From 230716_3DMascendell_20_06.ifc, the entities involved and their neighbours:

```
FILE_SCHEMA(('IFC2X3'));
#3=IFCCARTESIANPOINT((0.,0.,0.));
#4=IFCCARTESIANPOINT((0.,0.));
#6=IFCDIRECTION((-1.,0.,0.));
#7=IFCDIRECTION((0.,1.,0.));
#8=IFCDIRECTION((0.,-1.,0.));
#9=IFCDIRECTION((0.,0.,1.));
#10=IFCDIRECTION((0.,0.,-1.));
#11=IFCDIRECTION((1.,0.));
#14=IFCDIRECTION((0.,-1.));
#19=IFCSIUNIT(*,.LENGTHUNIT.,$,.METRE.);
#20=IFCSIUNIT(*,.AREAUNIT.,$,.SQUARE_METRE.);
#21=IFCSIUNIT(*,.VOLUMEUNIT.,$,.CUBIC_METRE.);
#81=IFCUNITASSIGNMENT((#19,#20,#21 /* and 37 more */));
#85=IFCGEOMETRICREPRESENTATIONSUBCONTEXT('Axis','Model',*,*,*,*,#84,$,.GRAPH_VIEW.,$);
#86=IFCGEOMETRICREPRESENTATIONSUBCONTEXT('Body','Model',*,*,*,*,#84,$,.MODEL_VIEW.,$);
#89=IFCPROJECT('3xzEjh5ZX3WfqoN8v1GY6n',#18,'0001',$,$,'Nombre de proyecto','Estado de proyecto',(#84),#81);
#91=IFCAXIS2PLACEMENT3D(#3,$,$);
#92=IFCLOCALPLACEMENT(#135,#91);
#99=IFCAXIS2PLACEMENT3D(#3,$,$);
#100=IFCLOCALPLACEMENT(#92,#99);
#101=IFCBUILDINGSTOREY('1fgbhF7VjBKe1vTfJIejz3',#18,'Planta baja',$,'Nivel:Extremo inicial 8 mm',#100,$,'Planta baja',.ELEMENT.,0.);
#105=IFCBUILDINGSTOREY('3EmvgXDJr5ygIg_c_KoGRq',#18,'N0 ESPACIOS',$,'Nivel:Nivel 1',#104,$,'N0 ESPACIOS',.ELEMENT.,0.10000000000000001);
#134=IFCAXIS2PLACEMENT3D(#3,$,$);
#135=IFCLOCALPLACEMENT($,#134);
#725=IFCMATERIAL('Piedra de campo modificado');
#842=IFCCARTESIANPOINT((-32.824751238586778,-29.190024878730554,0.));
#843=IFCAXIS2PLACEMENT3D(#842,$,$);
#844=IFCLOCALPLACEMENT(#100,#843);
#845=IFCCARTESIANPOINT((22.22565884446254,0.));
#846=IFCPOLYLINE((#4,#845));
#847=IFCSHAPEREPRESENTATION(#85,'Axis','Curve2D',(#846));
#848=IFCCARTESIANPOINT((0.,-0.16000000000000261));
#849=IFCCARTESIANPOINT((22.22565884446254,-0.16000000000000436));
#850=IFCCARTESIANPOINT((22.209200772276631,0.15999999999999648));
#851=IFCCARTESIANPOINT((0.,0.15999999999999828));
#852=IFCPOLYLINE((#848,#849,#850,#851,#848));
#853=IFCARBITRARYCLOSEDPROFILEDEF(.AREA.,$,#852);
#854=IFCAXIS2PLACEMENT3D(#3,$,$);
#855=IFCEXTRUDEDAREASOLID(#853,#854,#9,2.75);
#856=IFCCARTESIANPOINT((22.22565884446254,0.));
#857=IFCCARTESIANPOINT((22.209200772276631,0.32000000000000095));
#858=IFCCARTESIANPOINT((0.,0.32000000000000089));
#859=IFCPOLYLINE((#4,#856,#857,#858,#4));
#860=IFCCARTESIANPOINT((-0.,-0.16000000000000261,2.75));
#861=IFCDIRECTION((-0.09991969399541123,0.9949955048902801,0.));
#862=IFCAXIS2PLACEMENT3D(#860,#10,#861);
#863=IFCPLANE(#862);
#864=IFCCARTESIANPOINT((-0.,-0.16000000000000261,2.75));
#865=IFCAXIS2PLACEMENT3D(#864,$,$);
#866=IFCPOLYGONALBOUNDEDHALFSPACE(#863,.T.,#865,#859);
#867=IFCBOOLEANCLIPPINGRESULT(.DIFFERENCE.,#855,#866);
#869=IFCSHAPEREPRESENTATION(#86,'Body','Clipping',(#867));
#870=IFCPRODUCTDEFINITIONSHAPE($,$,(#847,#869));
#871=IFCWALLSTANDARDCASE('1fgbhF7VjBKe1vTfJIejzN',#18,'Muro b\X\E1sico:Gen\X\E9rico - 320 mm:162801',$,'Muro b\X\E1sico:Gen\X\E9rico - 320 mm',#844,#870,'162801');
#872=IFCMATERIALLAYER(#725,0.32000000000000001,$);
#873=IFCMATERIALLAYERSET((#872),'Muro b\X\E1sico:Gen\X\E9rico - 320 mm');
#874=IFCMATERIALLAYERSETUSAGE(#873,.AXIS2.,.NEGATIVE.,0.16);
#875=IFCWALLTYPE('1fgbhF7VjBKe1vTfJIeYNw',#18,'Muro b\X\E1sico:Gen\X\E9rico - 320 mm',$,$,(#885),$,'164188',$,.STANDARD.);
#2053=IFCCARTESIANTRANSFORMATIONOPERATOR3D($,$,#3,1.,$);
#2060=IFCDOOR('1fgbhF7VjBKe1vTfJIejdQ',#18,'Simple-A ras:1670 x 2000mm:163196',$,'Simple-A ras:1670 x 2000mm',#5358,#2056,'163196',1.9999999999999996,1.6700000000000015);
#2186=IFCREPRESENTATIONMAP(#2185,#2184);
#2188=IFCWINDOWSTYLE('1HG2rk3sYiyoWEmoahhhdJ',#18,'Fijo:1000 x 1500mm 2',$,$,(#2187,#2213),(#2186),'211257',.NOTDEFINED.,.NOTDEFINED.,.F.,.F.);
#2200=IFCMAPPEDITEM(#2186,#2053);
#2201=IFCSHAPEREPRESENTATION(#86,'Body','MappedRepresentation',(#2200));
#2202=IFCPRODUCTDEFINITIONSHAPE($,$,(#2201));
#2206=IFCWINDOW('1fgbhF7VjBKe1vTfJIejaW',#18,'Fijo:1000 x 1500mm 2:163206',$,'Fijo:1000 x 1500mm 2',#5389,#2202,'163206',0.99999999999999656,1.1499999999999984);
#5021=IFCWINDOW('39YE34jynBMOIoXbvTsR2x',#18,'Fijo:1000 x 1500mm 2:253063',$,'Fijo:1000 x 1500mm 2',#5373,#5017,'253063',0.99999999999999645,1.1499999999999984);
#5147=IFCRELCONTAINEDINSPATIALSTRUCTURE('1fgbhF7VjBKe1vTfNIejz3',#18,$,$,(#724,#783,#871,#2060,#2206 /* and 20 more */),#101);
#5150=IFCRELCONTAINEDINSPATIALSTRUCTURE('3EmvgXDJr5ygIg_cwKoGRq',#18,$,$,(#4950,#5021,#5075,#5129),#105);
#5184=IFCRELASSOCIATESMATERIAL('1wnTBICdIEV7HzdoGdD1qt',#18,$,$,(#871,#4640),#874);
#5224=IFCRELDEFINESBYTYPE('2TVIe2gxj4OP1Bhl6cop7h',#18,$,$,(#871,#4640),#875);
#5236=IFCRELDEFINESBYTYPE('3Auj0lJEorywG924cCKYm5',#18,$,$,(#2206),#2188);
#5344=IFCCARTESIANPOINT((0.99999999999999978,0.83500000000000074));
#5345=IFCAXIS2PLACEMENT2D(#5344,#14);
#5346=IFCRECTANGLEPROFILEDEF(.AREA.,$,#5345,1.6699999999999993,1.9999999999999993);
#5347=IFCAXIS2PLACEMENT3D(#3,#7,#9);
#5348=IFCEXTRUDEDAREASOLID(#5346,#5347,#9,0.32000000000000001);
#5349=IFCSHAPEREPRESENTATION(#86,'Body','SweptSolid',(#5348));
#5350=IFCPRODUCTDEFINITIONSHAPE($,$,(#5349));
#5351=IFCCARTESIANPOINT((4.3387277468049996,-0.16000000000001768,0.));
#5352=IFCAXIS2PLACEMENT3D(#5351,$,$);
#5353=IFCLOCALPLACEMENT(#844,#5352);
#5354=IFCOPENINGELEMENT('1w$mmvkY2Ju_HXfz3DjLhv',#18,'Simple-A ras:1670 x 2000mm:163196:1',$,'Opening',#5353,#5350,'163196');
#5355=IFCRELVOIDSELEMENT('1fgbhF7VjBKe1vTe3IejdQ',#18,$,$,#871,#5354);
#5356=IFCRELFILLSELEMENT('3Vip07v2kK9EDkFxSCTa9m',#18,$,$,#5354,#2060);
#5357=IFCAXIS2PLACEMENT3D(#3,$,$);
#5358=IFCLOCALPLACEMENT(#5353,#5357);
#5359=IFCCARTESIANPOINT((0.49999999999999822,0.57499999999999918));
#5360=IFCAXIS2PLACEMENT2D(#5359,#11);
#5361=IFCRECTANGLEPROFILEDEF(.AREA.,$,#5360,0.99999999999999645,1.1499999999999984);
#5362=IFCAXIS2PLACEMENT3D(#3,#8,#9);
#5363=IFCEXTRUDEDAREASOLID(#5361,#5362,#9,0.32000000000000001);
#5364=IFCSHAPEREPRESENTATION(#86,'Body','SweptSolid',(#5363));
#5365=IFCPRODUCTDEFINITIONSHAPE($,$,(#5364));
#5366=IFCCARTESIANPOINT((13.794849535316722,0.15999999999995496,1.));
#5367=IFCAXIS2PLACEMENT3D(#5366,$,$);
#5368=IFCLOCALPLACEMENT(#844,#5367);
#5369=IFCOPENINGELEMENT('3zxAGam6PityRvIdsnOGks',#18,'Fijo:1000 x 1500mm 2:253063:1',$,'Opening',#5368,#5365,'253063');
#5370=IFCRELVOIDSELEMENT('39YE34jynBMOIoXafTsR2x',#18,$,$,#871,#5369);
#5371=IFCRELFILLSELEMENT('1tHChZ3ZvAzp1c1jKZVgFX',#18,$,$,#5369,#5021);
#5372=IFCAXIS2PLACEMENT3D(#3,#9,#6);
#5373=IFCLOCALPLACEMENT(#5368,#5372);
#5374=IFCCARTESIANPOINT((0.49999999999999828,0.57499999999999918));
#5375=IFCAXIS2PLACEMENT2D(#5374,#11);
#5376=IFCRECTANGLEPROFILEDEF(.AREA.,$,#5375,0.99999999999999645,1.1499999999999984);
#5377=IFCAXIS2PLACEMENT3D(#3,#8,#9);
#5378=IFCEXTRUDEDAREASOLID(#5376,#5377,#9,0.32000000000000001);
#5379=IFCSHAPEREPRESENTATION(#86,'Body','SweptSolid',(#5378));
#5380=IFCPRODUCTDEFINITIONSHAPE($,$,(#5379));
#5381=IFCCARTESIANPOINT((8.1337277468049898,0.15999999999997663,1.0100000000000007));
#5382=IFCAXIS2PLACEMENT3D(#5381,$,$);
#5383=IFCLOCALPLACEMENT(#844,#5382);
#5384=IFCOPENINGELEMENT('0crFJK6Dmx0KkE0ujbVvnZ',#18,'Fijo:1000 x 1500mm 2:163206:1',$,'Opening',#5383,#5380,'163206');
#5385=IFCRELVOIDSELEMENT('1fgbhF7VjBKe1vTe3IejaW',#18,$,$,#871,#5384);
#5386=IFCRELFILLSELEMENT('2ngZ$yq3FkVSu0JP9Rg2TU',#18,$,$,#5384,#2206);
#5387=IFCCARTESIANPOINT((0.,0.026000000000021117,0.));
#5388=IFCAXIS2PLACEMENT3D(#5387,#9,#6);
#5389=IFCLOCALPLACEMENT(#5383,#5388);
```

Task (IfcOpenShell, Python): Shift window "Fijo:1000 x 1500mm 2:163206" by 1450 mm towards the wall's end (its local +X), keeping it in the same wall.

```python
import ifcopenshell
import ifcopenshell.api.geometry
import ifcopenshell.util.placement

model = ifcopenshell.open("230716_3DMascendell_20_06.ifc")

window = model.by_guid("1fgbhF7VjBKe1vTfJIejaW")
opening = window.FillsVoids[0].RelatingOpeningElement
wall = opening.VoidsElements[0].RelatingBuildingElement

wall_matrix = ifcopenshell.util.placement.get_local_placement(wall.ObjectPlacement)
shift = wall_matrix[:3, 0] * 1.45
before = ifcopenshell.util.placement.get_local_placement(window.ObjectPlacement)[:3, 3].copy()

# The window is placed relative to its opening, so it follows when the opening moves.
matrix = ifcopenshell.util.placement.get_local_placement(opening.ObjectPlacement)
matrix[:3, 3] += shift
ifcopenshell.api.geometry.edit_object_placement(
    model, product=opening, matrix=matrix, is_si=False, should_transform_children=True
)

after = ifcopenshell.util.placement.get_local_placement(window.ObjectPlacement)[:3, 3]
print("window moved by", (after - before).round(3) + 0.0)

model.write("230716_3DMascendell_20_06_rev.ifc")
```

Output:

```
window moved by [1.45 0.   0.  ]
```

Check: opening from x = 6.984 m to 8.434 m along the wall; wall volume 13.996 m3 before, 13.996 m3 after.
